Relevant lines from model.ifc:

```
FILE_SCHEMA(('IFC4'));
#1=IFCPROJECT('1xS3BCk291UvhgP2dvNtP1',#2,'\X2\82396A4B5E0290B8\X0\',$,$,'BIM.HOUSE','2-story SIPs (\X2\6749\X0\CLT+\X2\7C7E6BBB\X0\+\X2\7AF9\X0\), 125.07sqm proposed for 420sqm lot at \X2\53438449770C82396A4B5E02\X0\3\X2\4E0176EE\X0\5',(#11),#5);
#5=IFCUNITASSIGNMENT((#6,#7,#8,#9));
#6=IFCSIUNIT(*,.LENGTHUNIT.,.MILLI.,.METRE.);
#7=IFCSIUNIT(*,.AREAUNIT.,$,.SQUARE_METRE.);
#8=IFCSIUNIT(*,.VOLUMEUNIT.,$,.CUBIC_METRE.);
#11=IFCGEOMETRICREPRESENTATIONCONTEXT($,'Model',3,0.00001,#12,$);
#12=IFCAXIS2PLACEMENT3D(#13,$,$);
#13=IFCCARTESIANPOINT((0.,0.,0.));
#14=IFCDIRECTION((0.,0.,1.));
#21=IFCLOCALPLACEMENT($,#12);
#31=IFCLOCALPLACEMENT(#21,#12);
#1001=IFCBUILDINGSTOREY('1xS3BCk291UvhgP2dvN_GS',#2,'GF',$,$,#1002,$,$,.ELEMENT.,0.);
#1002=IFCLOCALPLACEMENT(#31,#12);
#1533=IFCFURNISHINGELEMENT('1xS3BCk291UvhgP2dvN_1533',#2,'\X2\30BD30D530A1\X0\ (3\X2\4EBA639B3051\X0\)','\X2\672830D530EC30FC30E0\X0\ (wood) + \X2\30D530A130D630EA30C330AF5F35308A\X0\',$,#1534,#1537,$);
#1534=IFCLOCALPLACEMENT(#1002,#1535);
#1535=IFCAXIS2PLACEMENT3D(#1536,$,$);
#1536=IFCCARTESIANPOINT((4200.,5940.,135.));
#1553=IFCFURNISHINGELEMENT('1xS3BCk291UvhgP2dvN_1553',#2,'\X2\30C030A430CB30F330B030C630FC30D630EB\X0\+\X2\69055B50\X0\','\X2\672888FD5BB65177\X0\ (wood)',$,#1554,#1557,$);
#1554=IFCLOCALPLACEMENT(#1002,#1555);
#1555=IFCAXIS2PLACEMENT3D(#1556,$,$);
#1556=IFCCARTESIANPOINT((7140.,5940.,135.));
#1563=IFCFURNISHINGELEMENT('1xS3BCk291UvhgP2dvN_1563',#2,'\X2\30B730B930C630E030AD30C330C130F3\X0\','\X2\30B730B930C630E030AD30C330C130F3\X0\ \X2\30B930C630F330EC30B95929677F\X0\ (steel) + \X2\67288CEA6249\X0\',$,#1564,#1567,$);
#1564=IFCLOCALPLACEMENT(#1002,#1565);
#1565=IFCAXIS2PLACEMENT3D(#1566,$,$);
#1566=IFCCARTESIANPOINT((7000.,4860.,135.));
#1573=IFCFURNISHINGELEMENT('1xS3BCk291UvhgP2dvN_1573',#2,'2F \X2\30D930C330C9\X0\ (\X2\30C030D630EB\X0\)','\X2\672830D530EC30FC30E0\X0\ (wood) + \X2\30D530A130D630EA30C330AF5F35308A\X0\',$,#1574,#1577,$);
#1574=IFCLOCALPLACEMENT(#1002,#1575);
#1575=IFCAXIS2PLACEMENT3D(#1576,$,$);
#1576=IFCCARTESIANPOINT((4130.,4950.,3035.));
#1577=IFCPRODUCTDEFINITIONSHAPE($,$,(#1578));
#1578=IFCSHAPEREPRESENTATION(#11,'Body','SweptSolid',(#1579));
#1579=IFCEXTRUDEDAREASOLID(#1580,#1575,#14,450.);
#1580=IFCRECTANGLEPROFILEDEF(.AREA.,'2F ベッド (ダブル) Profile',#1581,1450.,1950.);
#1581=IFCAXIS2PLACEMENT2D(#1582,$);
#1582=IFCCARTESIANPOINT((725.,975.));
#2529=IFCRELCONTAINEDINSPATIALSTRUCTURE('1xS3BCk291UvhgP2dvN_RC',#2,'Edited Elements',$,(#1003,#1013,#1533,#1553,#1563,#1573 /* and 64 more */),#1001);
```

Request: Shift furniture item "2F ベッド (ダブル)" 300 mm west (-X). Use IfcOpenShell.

```python
import ifcopenshell
import ifcopenshell.api.geometry
import ifcopenshell.util.placement
import ifcopenshell.util.unit

model = ifcopenshell.open("model.ifc")
unit_scale = ifcopenshell.util.unit.calculate_unit_scale(model)

item = model.by_id(1573)
matrix = ifcopenshell.util.placement.get_local_placement(item.ObjectPlacement)
matrix[0, 3] -= 0.3 / unit_scale
ifcopenshell.api.geometry.edit_object_placement(model, product=item, matrix=matrix, is_si=False)

print(ifcopenshell.util.placement.get_local_placement(item.ObjectPlacement).round(3) + 0.0)

model.write("model-out.ifc")
```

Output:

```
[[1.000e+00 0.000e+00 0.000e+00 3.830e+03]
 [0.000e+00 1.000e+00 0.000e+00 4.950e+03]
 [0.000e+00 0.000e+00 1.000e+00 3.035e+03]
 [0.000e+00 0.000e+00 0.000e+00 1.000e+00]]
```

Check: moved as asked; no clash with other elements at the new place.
